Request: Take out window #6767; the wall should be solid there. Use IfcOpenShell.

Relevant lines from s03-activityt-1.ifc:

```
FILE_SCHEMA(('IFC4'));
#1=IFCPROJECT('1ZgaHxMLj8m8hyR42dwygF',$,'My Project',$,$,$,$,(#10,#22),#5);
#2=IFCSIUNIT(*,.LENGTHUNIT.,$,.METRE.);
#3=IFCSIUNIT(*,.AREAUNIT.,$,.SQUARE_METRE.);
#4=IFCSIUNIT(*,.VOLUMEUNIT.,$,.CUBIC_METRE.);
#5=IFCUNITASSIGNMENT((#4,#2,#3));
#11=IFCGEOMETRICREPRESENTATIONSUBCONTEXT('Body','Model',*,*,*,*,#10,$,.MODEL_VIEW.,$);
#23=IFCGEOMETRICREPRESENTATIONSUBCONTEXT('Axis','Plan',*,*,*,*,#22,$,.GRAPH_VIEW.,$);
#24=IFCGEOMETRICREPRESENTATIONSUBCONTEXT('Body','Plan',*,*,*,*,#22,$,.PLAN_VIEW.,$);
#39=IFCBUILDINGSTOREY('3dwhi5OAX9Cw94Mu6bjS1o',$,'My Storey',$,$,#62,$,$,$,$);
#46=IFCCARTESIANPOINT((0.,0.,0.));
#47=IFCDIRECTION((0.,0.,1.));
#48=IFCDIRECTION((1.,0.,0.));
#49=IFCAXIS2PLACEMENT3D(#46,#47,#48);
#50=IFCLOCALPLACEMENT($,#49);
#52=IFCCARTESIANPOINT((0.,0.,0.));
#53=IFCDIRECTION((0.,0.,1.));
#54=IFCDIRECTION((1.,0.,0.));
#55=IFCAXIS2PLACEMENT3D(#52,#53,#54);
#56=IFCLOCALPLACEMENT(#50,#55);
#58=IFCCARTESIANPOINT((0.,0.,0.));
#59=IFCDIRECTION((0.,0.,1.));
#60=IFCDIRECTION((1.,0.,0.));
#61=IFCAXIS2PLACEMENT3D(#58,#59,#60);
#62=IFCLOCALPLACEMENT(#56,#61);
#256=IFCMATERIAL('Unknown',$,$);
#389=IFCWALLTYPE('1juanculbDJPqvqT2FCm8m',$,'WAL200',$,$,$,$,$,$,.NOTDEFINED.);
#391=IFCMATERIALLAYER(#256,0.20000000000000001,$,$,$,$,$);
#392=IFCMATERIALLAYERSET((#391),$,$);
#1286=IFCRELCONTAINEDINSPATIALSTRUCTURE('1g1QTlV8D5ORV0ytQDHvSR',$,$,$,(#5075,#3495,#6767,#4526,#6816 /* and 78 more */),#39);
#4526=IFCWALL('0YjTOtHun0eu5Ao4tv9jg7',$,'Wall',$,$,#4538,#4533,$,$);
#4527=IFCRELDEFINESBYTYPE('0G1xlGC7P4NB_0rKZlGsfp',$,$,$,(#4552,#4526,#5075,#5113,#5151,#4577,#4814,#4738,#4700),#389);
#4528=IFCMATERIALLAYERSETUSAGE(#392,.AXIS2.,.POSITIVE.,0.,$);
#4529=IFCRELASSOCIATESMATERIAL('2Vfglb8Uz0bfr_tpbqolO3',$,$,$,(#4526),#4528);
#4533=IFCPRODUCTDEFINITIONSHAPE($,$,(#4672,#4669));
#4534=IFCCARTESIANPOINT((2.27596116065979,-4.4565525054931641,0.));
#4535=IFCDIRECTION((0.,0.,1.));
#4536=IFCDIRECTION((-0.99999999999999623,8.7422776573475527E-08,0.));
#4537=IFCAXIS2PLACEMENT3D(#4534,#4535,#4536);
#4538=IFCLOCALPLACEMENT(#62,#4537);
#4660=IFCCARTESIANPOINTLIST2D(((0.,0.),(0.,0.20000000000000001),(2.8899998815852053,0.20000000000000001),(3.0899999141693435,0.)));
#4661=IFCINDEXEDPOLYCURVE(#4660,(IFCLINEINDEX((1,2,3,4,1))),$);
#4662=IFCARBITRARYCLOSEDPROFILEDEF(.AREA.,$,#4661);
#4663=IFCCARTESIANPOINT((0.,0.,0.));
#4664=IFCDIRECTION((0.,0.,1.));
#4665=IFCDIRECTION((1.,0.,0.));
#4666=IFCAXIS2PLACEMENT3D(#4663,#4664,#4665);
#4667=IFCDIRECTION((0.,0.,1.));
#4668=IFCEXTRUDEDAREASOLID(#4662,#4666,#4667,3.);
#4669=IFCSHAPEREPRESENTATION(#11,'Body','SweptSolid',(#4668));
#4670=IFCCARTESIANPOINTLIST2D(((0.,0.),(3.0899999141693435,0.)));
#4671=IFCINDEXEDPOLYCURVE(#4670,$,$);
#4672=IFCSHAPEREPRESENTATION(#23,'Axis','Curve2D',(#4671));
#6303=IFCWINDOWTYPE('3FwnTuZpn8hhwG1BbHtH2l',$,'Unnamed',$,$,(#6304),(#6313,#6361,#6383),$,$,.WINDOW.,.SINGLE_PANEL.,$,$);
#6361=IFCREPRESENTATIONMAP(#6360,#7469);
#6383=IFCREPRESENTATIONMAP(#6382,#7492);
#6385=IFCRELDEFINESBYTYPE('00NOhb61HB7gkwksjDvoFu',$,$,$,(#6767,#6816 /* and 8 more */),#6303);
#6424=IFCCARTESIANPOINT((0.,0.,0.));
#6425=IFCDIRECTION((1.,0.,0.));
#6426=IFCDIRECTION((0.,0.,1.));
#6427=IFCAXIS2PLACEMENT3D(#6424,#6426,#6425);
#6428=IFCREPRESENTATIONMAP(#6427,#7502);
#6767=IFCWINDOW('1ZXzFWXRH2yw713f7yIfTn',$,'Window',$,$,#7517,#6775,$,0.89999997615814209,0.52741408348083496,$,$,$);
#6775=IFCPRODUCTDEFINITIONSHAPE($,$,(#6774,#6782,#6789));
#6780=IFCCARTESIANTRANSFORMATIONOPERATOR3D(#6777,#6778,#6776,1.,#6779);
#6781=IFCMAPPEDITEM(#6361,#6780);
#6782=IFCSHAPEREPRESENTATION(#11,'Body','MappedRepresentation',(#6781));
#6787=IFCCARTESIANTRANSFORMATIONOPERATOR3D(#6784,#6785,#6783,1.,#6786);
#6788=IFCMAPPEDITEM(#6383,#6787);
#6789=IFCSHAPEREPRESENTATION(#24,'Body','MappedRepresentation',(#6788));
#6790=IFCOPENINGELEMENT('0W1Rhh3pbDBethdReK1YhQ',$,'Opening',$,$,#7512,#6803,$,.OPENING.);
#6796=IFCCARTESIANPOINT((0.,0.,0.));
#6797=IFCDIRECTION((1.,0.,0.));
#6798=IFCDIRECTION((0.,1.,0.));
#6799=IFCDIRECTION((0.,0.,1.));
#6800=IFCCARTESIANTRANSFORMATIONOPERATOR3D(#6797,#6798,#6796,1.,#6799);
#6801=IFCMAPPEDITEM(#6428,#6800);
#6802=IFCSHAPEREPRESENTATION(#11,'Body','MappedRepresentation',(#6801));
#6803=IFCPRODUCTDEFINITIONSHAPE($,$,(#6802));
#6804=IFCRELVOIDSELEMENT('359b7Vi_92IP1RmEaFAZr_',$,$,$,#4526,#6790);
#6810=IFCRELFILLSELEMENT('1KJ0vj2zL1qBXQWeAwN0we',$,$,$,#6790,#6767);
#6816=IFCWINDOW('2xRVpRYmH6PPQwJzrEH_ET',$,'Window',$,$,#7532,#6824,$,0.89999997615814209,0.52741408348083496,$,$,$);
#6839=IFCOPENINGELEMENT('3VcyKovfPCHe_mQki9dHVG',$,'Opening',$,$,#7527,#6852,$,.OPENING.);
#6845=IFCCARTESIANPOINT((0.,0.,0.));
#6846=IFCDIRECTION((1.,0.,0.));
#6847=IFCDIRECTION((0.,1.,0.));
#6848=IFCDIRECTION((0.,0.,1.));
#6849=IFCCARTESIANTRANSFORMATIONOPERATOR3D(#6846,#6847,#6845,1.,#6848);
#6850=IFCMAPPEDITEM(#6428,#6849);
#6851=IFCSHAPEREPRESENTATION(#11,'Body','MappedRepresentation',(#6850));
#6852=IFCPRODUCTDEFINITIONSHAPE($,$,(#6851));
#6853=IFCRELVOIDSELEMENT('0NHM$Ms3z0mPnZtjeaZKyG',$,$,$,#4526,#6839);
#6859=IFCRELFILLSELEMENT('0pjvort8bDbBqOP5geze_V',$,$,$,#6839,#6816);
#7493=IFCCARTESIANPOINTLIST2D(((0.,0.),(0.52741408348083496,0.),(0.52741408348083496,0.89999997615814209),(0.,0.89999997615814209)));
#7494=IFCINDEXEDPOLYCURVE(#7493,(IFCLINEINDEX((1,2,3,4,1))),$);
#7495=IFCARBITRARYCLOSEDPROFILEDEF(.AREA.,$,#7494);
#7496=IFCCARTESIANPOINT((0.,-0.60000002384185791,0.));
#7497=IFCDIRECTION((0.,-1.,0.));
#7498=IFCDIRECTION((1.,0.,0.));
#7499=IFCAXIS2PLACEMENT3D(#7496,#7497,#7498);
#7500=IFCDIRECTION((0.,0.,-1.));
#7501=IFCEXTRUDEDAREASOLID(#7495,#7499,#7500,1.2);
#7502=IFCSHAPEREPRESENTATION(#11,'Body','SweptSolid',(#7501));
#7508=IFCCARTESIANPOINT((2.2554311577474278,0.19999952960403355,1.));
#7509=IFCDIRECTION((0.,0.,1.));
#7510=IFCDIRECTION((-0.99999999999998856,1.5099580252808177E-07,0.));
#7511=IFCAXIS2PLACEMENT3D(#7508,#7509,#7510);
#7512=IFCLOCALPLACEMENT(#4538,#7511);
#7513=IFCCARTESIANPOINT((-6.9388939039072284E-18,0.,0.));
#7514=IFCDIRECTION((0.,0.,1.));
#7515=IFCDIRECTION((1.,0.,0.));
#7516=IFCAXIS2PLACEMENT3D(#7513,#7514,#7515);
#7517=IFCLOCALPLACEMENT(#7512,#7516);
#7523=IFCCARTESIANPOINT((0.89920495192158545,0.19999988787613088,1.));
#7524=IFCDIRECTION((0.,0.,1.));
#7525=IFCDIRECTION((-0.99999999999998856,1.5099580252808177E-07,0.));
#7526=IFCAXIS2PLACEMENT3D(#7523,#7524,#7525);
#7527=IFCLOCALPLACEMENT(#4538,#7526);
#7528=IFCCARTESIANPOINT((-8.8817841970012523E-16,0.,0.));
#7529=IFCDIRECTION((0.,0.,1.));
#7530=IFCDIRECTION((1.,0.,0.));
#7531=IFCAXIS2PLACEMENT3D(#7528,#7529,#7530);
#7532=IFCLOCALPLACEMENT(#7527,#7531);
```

```python
import ifcopenshell
import ifcopenshell.api.feature
import ifcopenshell.api.root
import ifcopenshell.geom
import ifcopenshell.util.shape

model = ifcopenshell.open("s03-activityt-1.ifc")
settings = ifcopenshell.geom.settings()


def volume(element):
    """Net volume in cubic metres, openings subtracted."""
    shape = ifcopenshell.geom.create_shape(settings, element)
    return ifcopenshell.util.shape.get_volume(shape.geometry)


window = model.by_guid("1ZXzFWXRH2yw713f7yIfTn")
opening = window.FillsVoids[0].RelatingOpeningElement
wall = opening.VoidsElements[0].RelatingBuildingElement
before = volume(wall)

ifcopenshell.api.root.remove_product(model, product=window)
ifcopenshell.api.feature.remove_feature(model, feature=opening)

after = volume(wall)

print(f"wall volume {before:.3f} -> {after:.3f} m3")

model.write("s03-activityt-1-out.ifc")
```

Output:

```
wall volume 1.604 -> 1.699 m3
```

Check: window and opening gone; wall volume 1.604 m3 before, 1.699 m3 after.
